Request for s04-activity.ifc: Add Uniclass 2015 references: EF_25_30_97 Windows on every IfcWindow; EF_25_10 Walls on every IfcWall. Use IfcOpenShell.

First a look at what the model holds.

```python
import ifcopenshell

model = ifcopenshell.open("s04-activity.ifc")
print(model.schema)
print("classifications:", [c.Name for c in model.by_type("IfcClassification")])
for ifc_class in ("IfcDoor", "IfcRoof", "IfcStair", "IfcWall", "IfcWindow"):
    print(ifc_class, len(model.by_type(ifc_class)))
```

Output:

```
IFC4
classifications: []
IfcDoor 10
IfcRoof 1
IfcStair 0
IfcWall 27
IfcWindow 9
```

```python
import ifcopenshell
import ifcopenshell.api.classification

model = ifcopenshell.open("s04-activity.ifc")

system = ifcopenshell.api.classification.add_classification(model, classification="Uniclass 2015")

codes = {
    "IfcWindow": ("EF_25_30_97", "Windows"),
    "IfcWall": ("EF_25_10", "Walls"),
}
for ifc_class, (code, name) in codes.items():
    products = model.by_type(ifc_class)
    ifcopenshell.api.classification.add_reference(
        model, products=products, classification=system, identification=code, name=name
    )
    print(code, len(products))

model.write("s04-activity-out.ifc")
```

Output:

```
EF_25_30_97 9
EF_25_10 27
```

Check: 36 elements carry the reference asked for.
